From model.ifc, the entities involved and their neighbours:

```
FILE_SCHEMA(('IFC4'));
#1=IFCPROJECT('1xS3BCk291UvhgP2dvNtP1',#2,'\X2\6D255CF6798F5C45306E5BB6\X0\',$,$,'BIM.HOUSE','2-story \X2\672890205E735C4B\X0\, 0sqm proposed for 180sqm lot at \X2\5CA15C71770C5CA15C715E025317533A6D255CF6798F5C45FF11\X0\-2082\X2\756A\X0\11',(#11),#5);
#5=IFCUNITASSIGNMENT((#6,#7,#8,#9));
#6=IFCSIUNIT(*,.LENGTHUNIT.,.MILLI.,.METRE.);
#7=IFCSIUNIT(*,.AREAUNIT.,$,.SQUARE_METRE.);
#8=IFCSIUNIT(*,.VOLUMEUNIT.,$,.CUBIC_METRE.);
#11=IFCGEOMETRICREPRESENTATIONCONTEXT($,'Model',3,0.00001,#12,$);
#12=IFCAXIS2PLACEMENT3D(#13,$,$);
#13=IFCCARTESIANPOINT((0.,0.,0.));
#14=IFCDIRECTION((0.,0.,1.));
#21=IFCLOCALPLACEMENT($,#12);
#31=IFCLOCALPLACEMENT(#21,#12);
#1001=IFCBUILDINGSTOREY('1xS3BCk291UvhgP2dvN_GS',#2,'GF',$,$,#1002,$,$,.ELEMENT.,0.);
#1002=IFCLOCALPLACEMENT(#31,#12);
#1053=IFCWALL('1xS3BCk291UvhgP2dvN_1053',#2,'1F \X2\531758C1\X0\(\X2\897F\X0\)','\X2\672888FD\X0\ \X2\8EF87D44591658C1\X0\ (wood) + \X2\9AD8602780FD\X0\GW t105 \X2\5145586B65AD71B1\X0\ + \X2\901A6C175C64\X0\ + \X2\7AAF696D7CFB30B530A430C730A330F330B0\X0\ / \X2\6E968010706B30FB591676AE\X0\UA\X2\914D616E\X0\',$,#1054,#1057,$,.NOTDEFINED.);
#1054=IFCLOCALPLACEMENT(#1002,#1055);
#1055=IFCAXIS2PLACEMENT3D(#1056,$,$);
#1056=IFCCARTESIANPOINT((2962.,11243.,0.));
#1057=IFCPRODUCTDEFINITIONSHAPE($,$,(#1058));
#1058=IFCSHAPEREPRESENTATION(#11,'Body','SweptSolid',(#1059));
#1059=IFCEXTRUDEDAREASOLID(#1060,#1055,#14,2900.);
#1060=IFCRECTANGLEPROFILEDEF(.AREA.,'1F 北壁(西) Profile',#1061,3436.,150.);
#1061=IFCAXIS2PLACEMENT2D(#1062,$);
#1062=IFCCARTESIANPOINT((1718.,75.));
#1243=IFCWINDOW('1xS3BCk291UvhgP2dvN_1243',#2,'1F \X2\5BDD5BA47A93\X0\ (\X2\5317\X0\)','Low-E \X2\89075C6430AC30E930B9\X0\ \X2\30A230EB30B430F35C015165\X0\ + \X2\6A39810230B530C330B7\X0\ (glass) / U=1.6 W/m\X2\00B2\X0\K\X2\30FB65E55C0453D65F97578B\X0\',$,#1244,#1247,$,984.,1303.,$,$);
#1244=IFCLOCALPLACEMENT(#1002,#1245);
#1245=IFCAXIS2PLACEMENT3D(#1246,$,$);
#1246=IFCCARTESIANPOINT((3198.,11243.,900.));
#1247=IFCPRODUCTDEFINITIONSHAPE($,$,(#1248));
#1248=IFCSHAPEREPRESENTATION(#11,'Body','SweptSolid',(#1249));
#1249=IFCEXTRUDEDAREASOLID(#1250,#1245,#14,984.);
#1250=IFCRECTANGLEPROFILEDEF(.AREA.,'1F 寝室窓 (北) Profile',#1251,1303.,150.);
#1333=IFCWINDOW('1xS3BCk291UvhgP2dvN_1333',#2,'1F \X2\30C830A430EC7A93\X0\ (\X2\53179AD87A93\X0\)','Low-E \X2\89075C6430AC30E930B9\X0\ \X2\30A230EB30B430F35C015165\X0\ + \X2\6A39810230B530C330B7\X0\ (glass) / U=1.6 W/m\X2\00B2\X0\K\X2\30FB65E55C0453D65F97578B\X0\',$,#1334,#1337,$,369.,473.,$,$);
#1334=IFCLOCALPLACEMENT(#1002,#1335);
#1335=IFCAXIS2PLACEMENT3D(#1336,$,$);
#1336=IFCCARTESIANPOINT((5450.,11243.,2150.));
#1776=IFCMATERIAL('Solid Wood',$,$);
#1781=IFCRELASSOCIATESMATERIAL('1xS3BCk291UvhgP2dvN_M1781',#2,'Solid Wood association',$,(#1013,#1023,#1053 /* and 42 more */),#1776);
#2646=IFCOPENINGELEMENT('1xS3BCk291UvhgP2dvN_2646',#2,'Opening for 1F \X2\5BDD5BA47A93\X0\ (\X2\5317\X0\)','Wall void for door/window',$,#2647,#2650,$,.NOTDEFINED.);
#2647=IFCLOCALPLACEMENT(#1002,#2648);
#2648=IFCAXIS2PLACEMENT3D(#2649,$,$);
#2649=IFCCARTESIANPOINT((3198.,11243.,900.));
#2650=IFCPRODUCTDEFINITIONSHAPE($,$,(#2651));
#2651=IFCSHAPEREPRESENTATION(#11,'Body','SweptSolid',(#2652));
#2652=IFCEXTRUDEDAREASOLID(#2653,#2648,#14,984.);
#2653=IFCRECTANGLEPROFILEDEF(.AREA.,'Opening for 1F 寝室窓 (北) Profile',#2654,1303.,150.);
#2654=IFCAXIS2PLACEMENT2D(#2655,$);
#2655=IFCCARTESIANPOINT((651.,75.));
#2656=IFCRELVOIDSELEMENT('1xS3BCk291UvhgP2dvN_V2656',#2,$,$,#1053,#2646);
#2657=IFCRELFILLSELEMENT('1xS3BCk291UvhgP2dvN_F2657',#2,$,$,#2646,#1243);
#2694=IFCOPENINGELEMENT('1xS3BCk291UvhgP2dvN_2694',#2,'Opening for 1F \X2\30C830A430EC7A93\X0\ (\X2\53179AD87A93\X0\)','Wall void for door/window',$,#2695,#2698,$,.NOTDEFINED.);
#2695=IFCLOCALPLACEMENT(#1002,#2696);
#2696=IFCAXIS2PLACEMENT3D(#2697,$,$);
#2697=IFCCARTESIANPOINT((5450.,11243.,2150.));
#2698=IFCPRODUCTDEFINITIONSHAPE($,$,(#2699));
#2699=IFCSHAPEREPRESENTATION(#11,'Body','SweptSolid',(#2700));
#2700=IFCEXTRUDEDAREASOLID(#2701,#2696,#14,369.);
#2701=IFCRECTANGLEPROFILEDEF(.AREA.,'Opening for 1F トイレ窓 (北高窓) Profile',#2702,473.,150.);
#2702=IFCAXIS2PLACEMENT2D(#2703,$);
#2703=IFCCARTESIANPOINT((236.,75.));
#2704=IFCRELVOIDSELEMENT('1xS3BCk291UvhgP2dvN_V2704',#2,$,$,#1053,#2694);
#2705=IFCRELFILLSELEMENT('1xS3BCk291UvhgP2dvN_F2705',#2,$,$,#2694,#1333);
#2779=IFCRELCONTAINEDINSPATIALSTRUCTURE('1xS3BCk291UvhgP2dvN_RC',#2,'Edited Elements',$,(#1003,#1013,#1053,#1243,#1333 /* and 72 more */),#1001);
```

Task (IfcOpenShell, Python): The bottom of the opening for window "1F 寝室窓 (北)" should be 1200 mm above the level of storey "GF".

```python
import numpy as np
import ifcopenshell
import ifcopenshell.api.geometry
import ifcopenshell.geom
import ifcopenshell.util.element
import ifcopenshell.util.placement
import ifcopenshell.util.shape
import ifcopenshell.util.unit

model = ifcopenshell.open("model.ifc")
unit_scale = ifcopenshell.util.unit.calculate_unit_scale(model)

window = model.by_id(1243)
opening = window.FillsVoids[0].RelatingOpeningElement
storey = ifcopenshell.util.element.get_container(window, ifc_class="IfcBuildingStorey")
level = ifcopenshell.util.placement.get_local_placement(storey.ObjectPlacement)[2, 3]

# The opening's origin need not be at the sill, so measure its lowest point.
shape = ifcopenshell.geom.create_shape(ifcopenshell.geom.settings(), opening)
bottom = ifcopenshell.util.shape.get_shape_bottom_elevation(shape, shape.geometry) / unit_scale
dz = level + 1.2 / unit_scale - bottom

shift = np.array([0.0, 0.0, dz])
# The window is not placed relative to its opening, so move both.
for product in (opening, window):
    matrix = ifcopenshell.util.placement.get_local_placement(product.ObjectPlacement)
    matrix[:3, 3] += shift
    ifcopenshell.api.geometry.edit_object_placement(model, product=product, matrix=matrix, is_si=False)

print(f"moved by {dz * unit_scale:+.3f} m")

model.write("model-out.ifc")
```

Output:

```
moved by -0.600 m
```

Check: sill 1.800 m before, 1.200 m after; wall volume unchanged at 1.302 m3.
